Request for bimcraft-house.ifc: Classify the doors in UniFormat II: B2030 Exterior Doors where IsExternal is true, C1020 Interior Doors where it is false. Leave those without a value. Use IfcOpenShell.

First a look at what the model holds.

```python
import ifcopenshell
import ifcopenshell.util.element

model = ifcopenshell.open("bimcraft-house.ifc")
print(model.schema)
print("classifications:", [c.Name for c in model.by_type("IfcClassification")])
values = [ifcopenshell.util.element.get_pset(e, "Pset_DoorCommon", "IsExternal") for e in model.by_type("IfcDoor")]
for value in (True, False, None):
    print("IsExternal", value, values.count(value))
```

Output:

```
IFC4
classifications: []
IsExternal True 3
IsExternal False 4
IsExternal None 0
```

```python
import ifcopenshell
import ifcopenshell.api.classification
import ifcopenshell.util.element

model = ifcopenshell.open("bimcraft-house.ifc")

system = ifcopenshell.api.classification.add_classification(model, classification="UniFormat II")

doors = model.by_type("IfcDoor")
external = {e: ifcopenshell.util.element.get_pset(e, "Pset_DoorCommon", "IsExternal") for e in doors}
for flag, code, name in ((True, "B2030", "Exterior Doors"), (False, "C1020", "Interior Doors")):
    products = [e for e in doors if external[e] is flag]
    ifcopenshell.api.classification.add_reference(
        model, products=products, classification=system, identification=code, name=name
    )
    print(code, len(products))

model.write("bimcraft-house_rev.ifc")
```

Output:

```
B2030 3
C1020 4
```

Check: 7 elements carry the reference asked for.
